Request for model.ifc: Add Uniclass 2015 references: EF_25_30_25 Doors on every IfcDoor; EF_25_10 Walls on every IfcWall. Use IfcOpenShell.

First a look at what the model holds.

```python
import ifcopenshell

model = ifcopenshell.open("model.ifc")
print(model.schema)
print("classifications:", [c.Name for c in model.by_type("IfcClassification")])
for ifc_class in ("IfcDoor", "IfcRoof", "IfcStair", "IfcWall", "IfcWindow"):
    print(ifc_class, len(model.by_type(ifc_class)))
```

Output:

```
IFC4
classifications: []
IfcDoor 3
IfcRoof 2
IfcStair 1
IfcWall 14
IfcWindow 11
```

```python
import ifcopenshell
import ifcopenshell.api.classification

model = ifcopenshell.open("model.ifc")

system = ifcopenshell.api.classification.add_classification(model, classification="Uniclass 2015")

codes = {
    "IfcDoor": ("EF_25_30_25", "Doors"),
    "IfcWall": ("EF_25_10", "Walls"),
}
for ifc_class, (code, name) in codes.items():
    products = model.by_type(ifc_class)
    ifcopenshell.api.classification.add_reference(
        model, products=products, classification=system, identification=code, name=name
    )
    print(code, len(products))

model.write("model_updated.ifc")
```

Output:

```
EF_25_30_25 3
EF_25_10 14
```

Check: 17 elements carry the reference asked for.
